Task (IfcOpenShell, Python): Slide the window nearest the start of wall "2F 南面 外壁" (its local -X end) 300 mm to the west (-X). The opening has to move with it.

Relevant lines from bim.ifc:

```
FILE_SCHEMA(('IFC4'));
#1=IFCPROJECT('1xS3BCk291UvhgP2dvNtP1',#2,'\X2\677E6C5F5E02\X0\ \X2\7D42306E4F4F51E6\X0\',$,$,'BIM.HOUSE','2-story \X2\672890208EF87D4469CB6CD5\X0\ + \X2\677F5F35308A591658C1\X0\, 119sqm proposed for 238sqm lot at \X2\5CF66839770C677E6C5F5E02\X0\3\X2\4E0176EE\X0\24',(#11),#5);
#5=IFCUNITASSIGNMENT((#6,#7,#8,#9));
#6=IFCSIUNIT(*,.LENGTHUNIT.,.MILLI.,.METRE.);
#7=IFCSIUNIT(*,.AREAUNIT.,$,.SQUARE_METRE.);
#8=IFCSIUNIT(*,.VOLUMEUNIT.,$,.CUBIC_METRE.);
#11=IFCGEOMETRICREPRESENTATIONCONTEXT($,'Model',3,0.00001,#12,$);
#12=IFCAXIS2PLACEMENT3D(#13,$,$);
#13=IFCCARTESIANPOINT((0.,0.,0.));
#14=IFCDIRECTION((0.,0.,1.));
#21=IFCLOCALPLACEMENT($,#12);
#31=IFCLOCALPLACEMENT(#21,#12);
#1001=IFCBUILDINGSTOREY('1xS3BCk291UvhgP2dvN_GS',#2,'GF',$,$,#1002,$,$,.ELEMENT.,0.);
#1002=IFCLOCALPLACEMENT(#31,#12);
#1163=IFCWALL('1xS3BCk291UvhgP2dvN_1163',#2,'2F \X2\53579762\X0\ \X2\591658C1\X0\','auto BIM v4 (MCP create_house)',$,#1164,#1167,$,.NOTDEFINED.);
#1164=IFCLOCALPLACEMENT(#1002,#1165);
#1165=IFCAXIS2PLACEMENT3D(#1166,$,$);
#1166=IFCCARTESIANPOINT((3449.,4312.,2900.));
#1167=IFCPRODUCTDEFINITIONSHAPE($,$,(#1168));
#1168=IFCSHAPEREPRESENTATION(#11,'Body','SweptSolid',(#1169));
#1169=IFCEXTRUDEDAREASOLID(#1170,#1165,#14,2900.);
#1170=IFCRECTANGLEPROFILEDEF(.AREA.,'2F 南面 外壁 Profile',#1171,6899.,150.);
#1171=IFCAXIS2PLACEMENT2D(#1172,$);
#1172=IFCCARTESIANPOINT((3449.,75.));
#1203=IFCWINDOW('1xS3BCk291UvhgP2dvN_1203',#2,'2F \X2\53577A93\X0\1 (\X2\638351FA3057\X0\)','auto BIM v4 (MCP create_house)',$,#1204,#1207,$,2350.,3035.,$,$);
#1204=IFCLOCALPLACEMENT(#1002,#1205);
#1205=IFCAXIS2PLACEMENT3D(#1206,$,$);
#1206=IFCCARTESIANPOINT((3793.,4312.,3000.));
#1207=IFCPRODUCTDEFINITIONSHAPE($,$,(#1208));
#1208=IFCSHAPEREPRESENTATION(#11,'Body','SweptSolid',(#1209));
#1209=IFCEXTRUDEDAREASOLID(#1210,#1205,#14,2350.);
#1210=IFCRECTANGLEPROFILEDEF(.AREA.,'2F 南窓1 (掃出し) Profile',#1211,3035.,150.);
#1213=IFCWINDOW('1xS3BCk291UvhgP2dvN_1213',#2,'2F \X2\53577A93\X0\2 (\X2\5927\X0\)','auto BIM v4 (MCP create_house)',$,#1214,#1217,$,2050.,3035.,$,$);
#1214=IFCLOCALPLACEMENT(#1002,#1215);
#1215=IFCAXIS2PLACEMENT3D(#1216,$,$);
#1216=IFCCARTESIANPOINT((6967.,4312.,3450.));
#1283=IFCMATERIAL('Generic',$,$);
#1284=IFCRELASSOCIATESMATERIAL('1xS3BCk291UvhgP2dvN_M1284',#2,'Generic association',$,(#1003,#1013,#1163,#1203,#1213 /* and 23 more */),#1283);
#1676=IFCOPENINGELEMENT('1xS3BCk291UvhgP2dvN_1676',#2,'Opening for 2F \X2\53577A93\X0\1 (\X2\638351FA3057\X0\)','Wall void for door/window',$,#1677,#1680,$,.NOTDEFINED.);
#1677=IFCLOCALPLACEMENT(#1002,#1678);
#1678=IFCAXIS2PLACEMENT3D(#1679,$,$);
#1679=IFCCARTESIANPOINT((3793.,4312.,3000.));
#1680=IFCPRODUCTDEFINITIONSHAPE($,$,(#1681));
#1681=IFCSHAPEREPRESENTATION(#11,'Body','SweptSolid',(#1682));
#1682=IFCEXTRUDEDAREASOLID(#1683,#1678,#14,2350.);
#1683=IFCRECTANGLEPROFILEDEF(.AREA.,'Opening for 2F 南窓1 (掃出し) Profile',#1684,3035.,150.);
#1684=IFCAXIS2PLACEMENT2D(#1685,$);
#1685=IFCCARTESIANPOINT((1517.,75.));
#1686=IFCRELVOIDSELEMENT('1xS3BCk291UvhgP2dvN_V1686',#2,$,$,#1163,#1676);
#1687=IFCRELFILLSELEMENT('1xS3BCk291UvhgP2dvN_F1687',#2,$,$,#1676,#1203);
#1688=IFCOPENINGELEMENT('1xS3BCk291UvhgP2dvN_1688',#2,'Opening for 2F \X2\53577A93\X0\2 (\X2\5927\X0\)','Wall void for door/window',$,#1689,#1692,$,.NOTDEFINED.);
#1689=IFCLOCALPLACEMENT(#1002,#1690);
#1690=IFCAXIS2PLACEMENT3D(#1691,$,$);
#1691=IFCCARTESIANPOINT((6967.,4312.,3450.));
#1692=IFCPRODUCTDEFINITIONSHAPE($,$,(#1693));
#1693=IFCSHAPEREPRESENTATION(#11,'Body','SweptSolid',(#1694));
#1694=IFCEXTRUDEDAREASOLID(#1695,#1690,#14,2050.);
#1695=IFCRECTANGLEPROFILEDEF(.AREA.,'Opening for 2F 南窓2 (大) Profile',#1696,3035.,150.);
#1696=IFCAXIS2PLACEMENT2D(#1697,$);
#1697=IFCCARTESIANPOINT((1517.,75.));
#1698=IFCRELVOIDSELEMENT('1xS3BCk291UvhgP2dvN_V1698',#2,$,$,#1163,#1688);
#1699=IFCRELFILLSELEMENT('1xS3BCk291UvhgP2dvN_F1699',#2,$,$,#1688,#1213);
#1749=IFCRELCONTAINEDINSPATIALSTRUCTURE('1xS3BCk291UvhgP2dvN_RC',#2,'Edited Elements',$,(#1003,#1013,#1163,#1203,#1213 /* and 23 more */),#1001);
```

```python
import ifcopenshell
import ifcopenshell.api.geometry
import ifcopenshell.util.placement
import ifcopenshell.util.unit

model = ifcopenshell.open("bim.ifc")
unit_scale = ifcopenshell.util.unit.calculate_unit_scale(model)

window = model.by_id(1203)
opening = window.FillsVoids[0].RelatingOpeningElement
wall = opening.VoidsElements[0].RelatingBuildingElement

wall_matrix = ifcopenshell.util.placement.get_local_placement(wall.ObjectPlacement)
shift = wall_matrix[:3, 0] * -0.3 / unit_scale
before = ifcopenshell.util.placement.get_local_placement(window.ObjectPlacement)[:3, 3].copy()

# The window is not placed relative to its opening, so move both.
for product in (opening, window):
    matrix = ifcopenshell.util.placement.get_local_placement(product.ObjectPlacement)
    matrix[:3, 3] += shift
    ifcopenshell.api.geometry.edit_object_placement(model, product=product, matrix=matrix, is_si=False)

after = ifcopenshell.util.placement.get_local_placement(window.ObjectPlacement)[:3, 3]
print("window moved by", (after - before).round(3) + 0.0)

model.write("bim_updated.ifc")
```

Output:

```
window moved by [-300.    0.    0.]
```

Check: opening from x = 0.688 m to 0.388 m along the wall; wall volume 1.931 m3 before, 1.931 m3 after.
